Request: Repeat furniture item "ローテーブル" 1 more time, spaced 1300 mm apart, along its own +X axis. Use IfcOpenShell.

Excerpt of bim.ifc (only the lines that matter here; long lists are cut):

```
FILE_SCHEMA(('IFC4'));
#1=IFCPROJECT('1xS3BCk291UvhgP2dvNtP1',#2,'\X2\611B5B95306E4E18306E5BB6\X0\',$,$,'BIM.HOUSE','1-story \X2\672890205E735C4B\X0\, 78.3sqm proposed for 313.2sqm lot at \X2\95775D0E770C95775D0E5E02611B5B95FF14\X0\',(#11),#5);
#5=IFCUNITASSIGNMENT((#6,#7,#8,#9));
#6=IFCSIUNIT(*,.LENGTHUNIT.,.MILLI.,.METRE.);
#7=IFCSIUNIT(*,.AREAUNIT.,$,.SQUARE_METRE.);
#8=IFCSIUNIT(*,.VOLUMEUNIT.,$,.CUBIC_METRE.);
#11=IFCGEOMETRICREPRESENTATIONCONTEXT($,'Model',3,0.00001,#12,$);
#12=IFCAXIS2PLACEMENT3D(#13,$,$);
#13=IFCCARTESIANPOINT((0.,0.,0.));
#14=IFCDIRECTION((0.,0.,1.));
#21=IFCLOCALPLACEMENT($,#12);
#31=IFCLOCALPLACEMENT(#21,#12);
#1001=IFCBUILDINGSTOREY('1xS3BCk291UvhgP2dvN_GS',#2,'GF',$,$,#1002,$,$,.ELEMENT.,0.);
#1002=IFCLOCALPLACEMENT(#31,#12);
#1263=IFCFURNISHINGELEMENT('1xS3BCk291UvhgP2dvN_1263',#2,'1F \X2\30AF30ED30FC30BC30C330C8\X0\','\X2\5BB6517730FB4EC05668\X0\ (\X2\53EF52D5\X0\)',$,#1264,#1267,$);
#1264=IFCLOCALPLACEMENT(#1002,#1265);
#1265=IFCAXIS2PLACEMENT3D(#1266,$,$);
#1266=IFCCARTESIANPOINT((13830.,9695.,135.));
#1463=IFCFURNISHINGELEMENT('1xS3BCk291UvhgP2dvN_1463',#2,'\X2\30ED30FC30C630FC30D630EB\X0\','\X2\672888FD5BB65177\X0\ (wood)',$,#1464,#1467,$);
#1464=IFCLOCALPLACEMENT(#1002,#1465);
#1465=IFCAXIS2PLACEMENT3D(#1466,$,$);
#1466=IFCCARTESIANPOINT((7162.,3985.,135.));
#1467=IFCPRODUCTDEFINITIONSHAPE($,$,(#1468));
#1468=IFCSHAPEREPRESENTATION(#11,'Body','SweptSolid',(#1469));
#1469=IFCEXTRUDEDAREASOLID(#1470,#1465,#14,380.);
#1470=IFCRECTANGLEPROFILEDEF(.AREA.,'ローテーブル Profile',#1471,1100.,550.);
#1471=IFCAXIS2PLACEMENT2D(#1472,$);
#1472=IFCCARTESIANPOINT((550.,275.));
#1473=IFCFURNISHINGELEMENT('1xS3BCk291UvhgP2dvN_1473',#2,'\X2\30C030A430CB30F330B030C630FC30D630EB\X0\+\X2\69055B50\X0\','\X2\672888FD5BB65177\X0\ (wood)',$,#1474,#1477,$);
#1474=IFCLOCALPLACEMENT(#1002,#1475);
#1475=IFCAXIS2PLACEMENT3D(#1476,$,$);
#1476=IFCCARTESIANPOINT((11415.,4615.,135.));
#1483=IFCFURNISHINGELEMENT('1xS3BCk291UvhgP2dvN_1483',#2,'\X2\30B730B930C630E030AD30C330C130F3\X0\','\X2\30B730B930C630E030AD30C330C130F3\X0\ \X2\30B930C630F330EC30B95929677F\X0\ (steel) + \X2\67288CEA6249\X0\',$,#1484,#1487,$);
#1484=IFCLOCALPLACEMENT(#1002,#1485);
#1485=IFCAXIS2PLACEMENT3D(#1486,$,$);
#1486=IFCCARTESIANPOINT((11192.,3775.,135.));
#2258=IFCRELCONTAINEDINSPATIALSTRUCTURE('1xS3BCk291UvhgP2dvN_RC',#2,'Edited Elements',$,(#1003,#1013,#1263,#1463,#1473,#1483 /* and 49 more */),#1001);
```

```python
import ifcopenshell
import ifcopenshell.api.geometry
import ifcopenshell.api.root
import ifcopenshell.util.element
import ifcopenshell.util.placement
import ifcopenshell.util.unit

model = ifcopenshell.open("bim.ifc")
unit_scale = ifcopenshell.util.unit.calculate_unit_scale(model)


def reuse_history(source, copy):
    """copy_class also copies each property set's owner history, people and application; keep the originals."""
    for rel in copy.IsDefinedBy:
        if rel.is_a("IfcRelDefinesByProperties") and (history := rel.RelatingPropertyDefinition.OwnerHistory):
            rel.RelatingPropertyDefinition.OwnerHistory = source.OwnerHistory
            ifcopenshell.util.element.remove_deep2(model, history)


source = model.by_id(1463)
base = ifcopenshell.util.placement.get_local_placement(source.ObjectPlacement)
step = base[:3, 0] * 1.3 / unit_scale

for i in range(1, 2):
    copy = ifcopenshell.api.root.copy_class(model, product=source)
    copy.Representation = ifcopenshell.util.element.copy_deep(
        model, source.Representation, exclude=["IfcGeometricRepresentationContext", "IfcRepresentationMap"]
    )
    reuse_history(source, copy)
    matrix = base.copy()
    matrix[:3, 3] += i * step
    print("added at", matrix[:3, 3].round(3) + 0.0)
    ifcopenshell.api.geometry.edit_object_placement(model, product=copy, matrix=matrix, is_si=False)

model.write("bim-out.ifc")
```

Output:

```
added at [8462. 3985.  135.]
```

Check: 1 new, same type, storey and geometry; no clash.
